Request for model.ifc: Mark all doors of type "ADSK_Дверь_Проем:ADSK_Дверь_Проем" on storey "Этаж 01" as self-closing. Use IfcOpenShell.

First a look at what the model holds.

```python
import ifcopenshell
import ifcopenshell.util.element

model = ifcopenshell.open("model.ifc")
print(model.schema)
storey = next(s for s in model.by_type("IfcBuildingStorey") if s.Name == "Этаж 01")
doors = [e for e in ifcopenshell.util.element.get_decomposition(storey) if e.is_a("IfcDoor")]
seen = {}
for e in doors:
    element_type = ifcopenshell.util.element.get_type(e)
    key = (element_type.Name if element_type != e and element_type else None, ifcopenshell.util.element.get_pset(e, "Pset_DoorCommon", "SelfClosing"))
    seen[key] = seen.get(key, 0) + 1
for (name, value), count in sorted(seen.items(), key=str):
    print(count, "x", name, "|", value)
```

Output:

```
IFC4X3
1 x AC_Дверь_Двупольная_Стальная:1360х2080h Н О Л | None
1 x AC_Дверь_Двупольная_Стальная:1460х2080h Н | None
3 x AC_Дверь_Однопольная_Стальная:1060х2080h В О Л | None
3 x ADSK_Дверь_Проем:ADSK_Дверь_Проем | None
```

```python
import ifcopenshell
import ifcopenshell.api.pset
import ifcopenshell.util.element

model = ifcopenshell.open("model.ifc")

storey = next(s for s in model.by_type("IfcBuildingStorey") if s.Name == "Этаж 01")
doors = [e for e in ifcopenshell.util.element.get_decomposition(storey) if e.is_a("IfcDoor")]

count = 0
for e in doors:
    element_type = ifcopenshell.util.element.get_type(e)
    if element_type in (None, e) or element_type.Name != "ADSK_Дверь_Проем:ADSK_Дверь_Проем":
        continue
    # add_pset returns the element's existing set when there is one.
    pset = ifcopenshell.api.pset.add_pset(model, product=e, name="Pset_DoorCommon")
    ifcopenshell.api.pset.edit_pset(model, pset=pset, properties={"SelfClosing": True})
    count += 1

print(count, "doors updated")

model.write("model_updated.ifc")
```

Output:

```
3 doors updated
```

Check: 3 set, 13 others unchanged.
